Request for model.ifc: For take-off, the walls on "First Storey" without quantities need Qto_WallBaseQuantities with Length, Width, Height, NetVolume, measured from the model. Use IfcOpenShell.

First a look at what the model holds.

```python
import ifcopenshell
import ifcopenshell.util.element
import ifcopenshell.util.unit

model = ifcopenshell.open("model.ifc")
print(model.schema)
for unit_type in ("LENGTHUNIT", "AREAUNIT", "VOLUMEUNIT"):
    print(unit_type, ifcopenshell.util.unit.calculate_unit_scale(model, unit_type))
storey = next(s for s in model.by_type("IfcBuildingStorey") if s.Name == "First Storey")
walls = [e for e in ifcopenshell.util.element.get_decomposition(storey) if e.is_a("IfcWall")]
for e in sorted(walls, key=lambda e: e.id()):
    print(e.id(), e.is_a(), e.Name, list(ifcopenshell.util.element.get_psets(e, qtos_only=True)), sep=" | ")
```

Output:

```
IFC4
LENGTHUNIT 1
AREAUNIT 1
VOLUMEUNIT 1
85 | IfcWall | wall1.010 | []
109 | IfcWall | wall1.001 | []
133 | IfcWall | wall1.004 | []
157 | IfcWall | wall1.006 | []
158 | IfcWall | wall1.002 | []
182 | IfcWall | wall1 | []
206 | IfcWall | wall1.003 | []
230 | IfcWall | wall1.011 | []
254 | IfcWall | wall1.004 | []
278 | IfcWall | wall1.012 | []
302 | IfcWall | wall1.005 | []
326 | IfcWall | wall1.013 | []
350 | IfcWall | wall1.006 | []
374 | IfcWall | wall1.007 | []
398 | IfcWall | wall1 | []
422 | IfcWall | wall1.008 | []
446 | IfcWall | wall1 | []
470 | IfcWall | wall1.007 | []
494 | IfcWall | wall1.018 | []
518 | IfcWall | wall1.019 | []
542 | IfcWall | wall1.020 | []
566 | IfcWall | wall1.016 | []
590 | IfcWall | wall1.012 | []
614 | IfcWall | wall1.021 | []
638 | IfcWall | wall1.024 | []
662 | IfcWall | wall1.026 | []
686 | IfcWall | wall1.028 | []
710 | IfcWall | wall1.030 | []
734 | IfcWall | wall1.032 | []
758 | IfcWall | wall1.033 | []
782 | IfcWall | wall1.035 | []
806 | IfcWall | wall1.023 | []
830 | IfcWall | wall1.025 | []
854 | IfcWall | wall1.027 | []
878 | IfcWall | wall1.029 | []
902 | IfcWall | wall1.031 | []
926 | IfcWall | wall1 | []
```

```python
import ifcopenshell
import ifcopenshell.api.pset
import ifcopenshell.geom
import ifcopenshell.util.element
import ifcopenshell.util.shape
import ifcopenshell.util.unit

model = ifcopenshell.open("model.ifc")
unit_scale = ifcopenshell.util.unit.calculate_unit_scale(model)
volume_scale = ifcopenshell.util.unit.calculate_unit_scale(model, "VOLUMEUNIT")
settings = ifcopenshell.geom.settings()

storey = next(s for s in model.by_type("IfcBuildingStorey") if s.Name == "First Storey")
walls = [e for e in ifcopenshell.util.element.get_decomposition(storey) if e.is_a("IfcWall")]

for e in sorted(walls, key=lambda e: e.id()):
    if ifcopenshell.util.element.get_psets(e, qtos_only=True, should_inherit=False):
        continue
    # Geometry comes back in metres, in the element's own axes.
    shape = ifcopenshell.geom.create_shape(settings, e)
    values = {
        "Length": ifcopenshell.util.shape.get_x(shape.geometry) / unit_scale,
        "Width": ifcopenshell.util.shape.get_y(shape.geometry) / unit_scale,
        "Height": ifcopenshell.util.shape.get_z(shape.geometry) / unit_scale,
        "NetVolume": ifcopenshell.util.shape.get_volume(shape.geometry) / volume_scale,
    }
    qto = ifcopenshell.api.pset.add_qto(model, product=e, name="Qto_WallBaseQuantities")
    ifcopenshell.api.pset.edit_qto(model, qto=qto, properties=values)
    print(e.id(), {k: round(v, 3) for k, v in values.items()})

model.write("model_v2.ifc")
```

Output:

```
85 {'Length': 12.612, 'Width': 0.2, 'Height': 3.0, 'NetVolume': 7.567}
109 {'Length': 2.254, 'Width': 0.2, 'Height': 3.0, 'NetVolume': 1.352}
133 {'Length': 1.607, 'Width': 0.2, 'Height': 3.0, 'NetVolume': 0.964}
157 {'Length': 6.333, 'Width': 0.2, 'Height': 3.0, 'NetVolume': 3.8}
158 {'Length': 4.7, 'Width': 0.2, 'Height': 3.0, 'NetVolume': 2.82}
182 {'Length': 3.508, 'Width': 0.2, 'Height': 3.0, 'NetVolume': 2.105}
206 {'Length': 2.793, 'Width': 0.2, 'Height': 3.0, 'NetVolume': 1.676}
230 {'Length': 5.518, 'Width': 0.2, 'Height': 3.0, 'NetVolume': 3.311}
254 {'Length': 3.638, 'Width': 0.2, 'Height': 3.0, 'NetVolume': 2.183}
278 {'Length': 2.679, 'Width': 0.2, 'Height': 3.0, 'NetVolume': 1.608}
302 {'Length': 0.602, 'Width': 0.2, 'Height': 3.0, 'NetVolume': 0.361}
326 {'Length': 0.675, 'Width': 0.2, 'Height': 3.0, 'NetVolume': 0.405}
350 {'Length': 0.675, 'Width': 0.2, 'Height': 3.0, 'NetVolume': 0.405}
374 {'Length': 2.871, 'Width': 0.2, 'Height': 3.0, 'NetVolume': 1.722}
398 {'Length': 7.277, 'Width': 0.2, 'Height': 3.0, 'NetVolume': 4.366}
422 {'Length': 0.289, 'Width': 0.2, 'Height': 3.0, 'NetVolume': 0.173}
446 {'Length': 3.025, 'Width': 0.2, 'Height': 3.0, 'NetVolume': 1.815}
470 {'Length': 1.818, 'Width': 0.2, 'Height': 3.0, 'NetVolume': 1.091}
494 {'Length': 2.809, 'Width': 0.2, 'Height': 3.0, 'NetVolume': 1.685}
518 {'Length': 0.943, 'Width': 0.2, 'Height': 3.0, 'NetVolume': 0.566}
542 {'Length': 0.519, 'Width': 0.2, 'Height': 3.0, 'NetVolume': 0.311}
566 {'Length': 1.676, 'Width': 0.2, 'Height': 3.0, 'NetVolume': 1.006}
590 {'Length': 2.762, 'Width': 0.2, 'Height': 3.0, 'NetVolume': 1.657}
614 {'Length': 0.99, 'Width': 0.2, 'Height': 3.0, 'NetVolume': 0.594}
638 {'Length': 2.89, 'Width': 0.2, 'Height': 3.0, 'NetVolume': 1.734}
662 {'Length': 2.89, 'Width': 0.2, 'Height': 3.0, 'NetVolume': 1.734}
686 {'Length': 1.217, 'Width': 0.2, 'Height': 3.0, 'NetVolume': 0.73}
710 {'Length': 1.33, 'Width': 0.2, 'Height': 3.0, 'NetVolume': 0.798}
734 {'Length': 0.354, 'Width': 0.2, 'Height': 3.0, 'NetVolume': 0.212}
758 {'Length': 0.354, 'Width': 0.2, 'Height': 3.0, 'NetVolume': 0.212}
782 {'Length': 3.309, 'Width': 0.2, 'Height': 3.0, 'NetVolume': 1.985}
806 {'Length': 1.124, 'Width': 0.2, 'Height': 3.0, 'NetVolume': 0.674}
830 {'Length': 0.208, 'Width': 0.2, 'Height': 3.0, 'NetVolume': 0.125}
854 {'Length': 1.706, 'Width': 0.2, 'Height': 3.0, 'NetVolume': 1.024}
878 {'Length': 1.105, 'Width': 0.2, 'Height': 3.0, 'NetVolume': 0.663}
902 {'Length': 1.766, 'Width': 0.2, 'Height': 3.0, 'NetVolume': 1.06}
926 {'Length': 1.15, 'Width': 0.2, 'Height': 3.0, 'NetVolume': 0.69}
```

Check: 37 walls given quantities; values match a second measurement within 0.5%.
